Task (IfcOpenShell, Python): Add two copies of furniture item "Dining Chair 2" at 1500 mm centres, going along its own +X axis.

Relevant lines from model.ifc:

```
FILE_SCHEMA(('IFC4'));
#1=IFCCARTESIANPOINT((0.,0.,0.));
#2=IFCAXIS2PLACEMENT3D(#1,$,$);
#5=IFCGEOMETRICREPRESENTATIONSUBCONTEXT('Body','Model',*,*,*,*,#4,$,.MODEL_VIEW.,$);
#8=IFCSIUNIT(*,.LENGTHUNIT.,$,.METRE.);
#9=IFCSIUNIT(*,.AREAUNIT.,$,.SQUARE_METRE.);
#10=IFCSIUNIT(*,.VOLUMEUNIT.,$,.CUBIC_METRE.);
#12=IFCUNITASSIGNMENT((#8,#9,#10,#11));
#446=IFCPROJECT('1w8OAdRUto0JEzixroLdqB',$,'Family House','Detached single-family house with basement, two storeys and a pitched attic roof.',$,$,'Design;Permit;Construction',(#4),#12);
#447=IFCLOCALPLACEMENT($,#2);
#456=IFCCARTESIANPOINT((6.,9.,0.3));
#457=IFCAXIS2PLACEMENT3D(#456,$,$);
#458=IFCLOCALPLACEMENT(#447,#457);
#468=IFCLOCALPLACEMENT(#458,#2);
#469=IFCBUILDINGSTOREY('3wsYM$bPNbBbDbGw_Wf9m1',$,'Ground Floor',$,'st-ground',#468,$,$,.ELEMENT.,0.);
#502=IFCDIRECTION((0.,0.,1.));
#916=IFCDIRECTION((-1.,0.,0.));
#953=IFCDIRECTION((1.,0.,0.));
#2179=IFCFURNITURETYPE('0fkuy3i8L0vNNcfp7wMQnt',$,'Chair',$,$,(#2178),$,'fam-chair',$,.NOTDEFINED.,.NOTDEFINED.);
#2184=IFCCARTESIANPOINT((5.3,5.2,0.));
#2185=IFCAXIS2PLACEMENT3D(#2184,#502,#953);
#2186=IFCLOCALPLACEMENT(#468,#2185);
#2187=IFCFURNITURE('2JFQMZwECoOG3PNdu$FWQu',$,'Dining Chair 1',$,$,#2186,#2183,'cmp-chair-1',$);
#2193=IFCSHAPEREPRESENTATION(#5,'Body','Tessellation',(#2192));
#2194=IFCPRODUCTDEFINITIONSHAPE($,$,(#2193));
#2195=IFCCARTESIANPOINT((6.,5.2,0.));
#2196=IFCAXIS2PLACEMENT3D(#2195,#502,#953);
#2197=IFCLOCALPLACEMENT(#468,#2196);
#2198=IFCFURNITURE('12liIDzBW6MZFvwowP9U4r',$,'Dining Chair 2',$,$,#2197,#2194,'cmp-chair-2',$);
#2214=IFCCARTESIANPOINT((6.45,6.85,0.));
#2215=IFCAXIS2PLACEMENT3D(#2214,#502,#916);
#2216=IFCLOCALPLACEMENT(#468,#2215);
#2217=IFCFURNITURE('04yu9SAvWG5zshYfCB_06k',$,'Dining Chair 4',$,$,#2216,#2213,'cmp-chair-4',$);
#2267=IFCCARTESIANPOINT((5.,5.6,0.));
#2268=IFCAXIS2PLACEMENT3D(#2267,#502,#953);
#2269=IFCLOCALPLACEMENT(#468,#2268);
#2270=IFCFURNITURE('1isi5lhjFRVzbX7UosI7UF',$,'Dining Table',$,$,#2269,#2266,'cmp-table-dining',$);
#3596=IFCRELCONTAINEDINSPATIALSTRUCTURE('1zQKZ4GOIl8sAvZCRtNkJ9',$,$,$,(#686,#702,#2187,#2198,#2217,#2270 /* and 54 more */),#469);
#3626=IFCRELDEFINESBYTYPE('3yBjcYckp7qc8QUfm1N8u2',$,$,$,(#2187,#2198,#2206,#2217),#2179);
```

```python
import ifcopenshell
import ifcopenshell.api.geometry
import ifcopenshell.api.root
import ifcopenshell.util.element
import ifcopenshell.util.placement
import ifcopenshell.util.unit

model = ifcopenshell.open("model.ifc")
unit_scale = ifcopenshell.util.unit.calculate_unit_scale(model)

source = model.by_guid("12liIDzBW6MZFvwowP9U4r")
base = ifcopenshell.util.placement.get_local_placement(source.ObjectPlacement)
step = base[:3, 0] * 1.5 / unit_scale

for i in range(1, 3):
    copy = ifcopenshell.api.root.copy_class(model, product=source)
    copy.Representation = ifcopenshell.util.element.copy_deep(
        model, source.Representation, exclude=["IfcGeometricRepresentationContext", "IfcRepresentationMap"]
    )
    copy.Tag = None
    matrix = base.copy()
    matrix[:3, 3] += i * step
    print("added at", matrix[:3, 3].round(3) + 0.0)
    ifcopenshell.api.geometry.edit_object_placement(model, product=copy, matrix=matrix, is_si=False)

model.write("model_updated.ifc")
```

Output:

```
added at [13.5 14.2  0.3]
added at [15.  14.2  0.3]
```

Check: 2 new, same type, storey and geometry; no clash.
